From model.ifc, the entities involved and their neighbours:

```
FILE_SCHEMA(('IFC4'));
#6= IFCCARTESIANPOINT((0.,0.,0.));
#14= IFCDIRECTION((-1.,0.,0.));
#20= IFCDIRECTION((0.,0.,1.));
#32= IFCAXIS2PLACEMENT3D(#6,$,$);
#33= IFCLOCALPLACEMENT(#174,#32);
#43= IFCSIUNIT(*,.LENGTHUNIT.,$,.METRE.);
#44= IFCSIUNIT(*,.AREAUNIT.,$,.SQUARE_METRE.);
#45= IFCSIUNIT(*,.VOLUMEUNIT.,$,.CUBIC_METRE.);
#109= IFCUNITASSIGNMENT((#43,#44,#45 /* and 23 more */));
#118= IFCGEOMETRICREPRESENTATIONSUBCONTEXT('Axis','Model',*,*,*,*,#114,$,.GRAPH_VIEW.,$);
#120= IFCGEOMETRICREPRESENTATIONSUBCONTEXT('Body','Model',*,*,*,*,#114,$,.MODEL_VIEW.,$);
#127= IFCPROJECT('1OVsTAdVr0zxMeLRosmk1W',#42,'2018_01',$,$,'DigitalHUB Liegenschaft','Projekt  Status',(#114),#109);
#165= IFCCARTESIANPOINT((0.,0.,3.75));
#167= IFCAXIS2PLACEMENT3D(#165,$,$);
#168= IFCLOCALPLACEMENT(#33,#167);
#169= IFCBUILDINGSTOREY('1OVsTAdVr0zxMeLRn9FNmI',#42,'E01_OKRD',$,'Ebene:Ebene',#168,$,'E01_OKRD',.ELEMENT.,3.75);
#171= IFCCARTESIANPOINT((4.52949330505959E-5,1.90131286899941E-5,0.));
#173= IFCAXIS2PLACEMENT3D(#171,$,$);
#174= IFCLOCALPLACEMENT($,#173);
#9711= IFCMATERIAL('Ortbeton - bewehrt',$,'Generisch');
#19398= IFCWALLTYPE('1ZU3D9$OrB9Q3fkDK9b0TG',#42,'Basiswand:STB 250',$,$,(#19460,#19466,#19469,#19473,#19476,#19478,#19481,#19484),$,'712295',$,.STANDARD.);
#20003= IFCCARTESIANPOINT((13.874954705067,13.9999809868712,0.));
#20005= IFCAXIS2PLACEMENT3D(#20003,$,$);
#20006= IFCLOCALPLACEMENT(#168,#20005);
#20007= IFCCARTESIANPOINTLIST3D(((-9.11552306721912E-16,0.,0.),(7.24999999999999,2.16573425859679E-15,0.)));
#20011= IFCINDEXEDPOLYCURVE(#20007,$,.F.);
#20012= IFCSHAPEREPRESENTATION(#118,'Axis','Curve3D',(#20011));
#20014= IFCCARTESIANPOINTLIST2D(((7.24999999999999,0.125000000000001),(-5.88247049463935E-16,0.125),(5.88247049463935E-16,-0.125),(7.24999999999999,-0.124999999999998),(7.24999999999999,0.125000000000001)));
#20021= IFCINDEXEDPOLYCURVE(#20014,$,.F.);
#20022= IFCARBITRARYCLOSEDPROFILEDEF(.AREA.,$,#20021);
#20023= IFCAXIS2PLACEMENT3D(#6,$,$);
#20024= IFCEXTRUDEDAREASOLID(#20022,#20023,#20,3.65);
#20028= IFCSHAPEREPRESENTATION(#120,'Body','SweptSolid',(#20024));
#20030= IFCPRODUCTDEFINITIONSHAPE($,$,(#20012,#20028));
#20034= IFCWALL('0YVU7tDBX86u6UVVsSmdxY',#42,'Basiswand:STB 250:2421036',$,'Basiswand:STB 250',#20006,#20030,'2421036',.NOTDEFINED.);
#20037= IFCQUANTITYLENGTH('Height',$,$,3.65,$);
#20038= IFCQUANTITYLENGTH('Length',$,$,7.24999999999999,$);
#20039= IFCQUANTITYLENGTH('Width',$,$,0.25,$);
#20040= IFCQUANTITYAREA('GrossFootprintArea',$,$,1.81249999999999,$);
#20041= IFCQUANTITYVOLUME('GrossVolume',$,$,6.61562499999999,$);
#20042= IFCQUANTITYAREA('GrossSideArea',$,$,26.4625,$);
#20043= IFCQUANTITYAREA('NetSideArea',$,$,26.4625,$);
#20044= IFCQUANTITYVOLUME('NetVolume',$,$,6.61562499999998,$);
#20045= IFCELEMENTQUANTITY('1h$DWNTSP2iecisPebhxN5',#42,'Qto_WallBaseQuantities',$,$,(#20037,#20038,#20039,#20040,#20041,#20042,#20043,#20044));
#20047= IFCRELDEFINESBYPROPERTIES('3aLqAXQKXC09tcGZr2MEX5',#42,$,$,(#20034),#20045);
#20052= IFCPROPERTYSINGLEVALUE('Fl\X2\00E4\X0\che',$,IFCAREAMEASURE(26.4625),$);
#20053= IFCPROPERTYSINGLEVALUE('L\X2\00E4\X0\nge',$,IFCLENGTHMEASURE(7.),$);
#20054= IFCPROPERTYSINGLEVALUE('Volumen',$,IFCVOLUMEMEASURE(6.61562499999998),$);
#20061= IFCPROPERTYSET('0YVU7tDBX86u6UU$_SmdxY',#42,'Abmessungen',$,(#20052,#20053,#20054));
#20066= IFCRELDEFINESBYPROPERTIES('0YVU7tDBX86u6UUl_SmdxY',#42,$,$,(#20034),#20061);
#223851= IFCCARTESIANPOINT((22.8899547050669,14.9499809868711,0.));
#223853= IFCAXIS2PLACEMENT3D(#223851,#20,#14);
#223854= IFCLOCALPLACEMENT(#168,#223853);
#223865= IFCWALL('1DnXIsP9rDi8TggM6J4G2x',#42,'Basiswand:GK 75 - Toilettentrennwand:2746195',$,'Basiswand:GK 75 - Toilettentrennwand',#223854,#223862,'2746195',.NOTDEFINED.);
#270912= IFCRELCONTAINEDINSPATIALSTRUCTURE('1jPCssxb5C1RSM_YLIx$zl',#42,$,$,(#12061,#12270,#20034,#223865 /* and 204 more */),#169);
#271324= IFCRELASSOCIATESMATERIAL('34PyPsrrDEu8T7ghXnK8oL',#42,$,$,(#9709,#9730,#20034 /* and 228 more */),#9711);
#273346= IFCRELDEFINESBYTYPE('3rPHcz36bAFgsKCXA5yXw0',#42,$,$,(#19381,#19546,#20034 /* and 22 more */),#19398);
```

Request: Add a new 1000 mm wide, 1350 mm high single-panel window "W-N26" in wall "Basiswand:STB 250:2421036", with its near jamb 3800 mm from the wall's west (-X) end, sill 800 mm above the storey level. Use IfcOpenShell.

```python
import numpy as np
import ifcopenshell
import ifcopenshell.api.feature
import ifcopenshell.api.geometry
import ifcopenshell.api.pset
import ifcopenshell.api.root
import ifcopenshell.api.spatial
import ifcopenshell.geom
import ifcopenshell.util.element
import ifcopenshell.util.placement
import ifcopenshell.util.representation
import ifcopenshell.util.shape
import ifcopenshell.util.unit

model = ifcopenshell.open("model.ifc")
unit_scale = ifcopenshell.util.unit.calculate_unit_scale(model)
area_scale = ifcopenshell.util.unit.calculate_unit_scale(model, "AREAUNIT")
volume_scale = ifcopenshell.util.unit.calculate_unit_scale(model, "VOLUMEUNIT")
settings = ifcopenshell.geom.settings()


def volume(element):
    """Net volume in cubic metres, openings subtracted."""
    shape = ifcopenshell.geom.create_shape(settings, element)
    return ifcopenshell.util.shape.get_volume(shape.geometry)


wall = model.by_id(20034)
storey = ifcopenshell.util.element.get_container(wall, ifc_class="IfcBuildingStorey")
context = ifcopenshell.util.representation.get_context(model, "Model", "Body", "MODEL_VIEW")
before = volume(wall)

width, height, from_end, sill = 1, 1.35, 3.8, 0.8  # metres

# The wall runs along its own X axis, and the end named is its -X end.
wall_shape = ifcopenshell.geom.create_shape(settings, wall)
x, y, z = ifcopenshell.util.shape.get_vertices(wall_shape.geometry).T
start = x.min() + from_end
face, thickness = float(y.min()), float(y.max() - y.min())
wall_matrix = ifcopenshell.util.placement.get_local_placement(wall.ObjectPlacement)
level = ifcopenshell.util.placement.get_local_placement(storey.ObjectPlacement)[2, 3]


def in_wall(x, y):
    """Placement at x, y metres in the wall's axes, at sill height."""
    matrix = wall_matrix.copy()
    matrix[:, 3] = wall_matrix @ np.array([x / unit_scale, y / unit_scale, 0.0, 1.0])
    matrix[2, 3] = level + sill / unit_scale
    return matrix


# Opening: a box that overshoots both wall faces by 50 mm.
opening = ifcopenshell.api.root.create_entity(model, ifc_class="IfcOpeningElement", predefined_type="OPENING")
box = ifcopenshell.api.geometry.add_wall_representation(
    model, context=context, length=width, height=height, thickness=thickness + 0.1
)
ifcopenshell.api.geometry.assign_representation(model, product=opening, representation=box)
ifcopenshell.api.geometry.edit_object_placement(model, product=opening, matrix=in_wall(start, face - 0.05), is_si=False)
ifcopenshell.api.feature.add_feature(model, feature=opening, element=wall)

window = ifcopenshell.api.root.create_entity(model, ifc_class="IfcWindow", name="W-N26", predefined_type="WINDOW")
window.OverallWidth, window.OverallHeight = width / unit_scale, height / unit_scale
window.PartitioningType = "SINGLE_PANEL"
body = ifcopenshell.api.geometry.add_window_representation(
    model,
    context=context,
    overall_width=window.OverallWidth,
    overall_height=window.OverallHeight,
    partition_type="SINGLE_PANEL",
)
ifcopenshell.api.geometry.assign_representation(model, product=window, representation=body)
ifcopenshell.api.spatial.assign_container(model, products=[window], relating_structure=storey)
ifcopenshell.api.feature.add_filling(model, opening=opening, element=window)

# Centre the window in the wall's thickness.
ifcopenshell.api.geometry.edit_object_placement(model, product=window, matrix=in_wall(start, face), is_si=False)
window_shape = ifcopenshell.geom.create_shape(settings, window)
depth = ifcopenshell.util.shape.get_vertices(window_shape.geometry)[:, 1]
offset = face + thickness / 2 - (depth.min() + depth.max()) / 2
ifcopenshell.api.geometry.edit_object_placement(model, product=window, matrix=in_wall(start, offset), is_si=False)

after = volume(wall)

# Update the wall's stored quantities.
qto = model.by_id(ifcopenshell.util.element.get_pset(wall, "Qto_WallBaseQuantities", should_inherit=False)["id"])
ifcopenshell.api.pset.edit_qto(model, qto=qto, properties={
    "NetSideArea": after / thickness / area_scale,
    "NetVolume": after / volume_scale,
})
pset = model.by_id(ifcopenshell.util.element.get_pset(wall, "Abmessungen", should_inherit=False)["id"])
ifcopenshell.api.pset.edit_pset(model, pset=pset, properties={
    "Fläche": model.create_entity("IfcAreaMeasure", after / thickness / area_scale),
    "Volumen": model.create_entity("IfcVolumeMeasure", after / volume_scale),
})

print(f"wall volume {before:.3f} -> {after:.3f} m3")

model.write("model-out.ifc")
```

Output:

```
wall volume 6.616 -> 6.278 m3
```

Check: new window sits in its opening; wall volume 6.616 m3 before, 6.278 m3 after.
